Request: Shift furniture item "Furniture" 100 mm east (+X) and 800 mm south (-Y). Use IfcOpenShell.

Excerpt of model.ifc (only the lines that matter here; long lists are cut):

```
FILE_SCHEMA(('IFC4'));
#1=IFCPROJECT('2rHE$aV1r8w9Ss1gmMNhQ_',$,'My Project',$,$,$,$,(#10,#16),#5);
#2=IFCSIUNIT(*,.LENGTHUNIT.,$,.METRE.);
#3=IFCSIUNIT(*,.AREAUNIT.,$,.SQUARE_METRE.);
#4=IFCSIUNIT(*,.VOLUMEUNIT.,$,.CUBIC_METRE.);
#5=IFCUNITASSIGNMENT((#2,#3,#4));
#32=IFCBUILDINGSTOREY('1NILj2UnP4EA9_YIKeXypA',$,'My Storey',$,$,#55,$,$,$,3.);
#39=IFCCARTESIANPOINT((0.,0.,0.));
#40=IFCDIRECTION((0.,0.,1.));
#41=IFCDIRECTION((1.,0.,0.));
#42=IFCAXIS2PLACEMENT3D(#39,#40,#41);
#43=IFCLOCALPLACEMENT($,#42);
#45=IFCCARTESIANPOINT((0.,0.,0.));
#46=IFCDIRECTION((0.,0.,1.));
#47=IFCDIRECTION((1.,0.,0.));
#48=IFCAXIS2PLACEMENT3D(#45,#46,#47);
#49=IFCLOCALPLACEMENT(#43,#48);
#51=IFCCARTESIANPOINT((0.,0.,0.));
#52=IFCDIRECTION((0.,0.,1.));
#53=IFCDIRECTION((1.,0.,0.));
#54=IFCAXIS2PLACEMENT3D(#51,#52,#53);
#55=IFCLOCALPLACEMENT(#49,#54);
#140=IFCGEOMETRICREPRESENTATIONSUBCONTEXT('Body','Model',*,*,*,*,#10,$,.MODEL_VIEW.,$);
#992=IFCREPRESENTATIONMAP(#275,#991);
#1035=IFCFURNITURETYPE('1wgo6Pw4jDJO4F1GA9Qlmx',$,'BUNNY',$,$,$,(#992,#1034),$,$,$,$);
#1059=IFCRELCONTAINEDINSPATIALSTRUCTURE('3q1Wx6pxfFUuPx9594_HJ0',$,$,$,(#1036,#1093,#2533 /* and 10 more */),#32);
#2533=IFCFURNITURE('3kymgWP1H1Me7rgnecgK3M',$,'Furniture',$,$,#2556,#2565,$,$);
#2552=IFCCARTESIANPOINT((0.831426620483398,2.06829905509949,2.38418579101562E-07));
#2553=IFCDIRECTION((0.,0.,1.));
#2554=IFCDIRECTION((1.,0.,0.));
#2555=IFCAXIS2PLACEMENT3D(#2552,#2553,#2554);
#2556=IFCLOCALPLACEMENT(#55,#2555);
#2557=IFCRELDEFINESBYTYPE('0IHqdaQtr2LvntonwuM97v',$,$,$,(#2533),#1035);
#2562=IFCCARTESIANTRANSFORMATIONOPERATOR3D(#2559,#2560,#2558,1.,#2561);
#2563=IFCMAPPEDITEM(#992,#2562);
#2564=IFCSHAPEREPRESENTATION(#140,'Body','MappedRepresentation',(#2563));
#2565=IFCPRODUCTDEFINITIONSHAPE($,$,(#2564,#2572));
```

```python
import ifcopenshell
import ifcopenshell.api.geometry
import ifcopenshell.util.placement

model = ifcopenshell.open("model.ifc")

item = model.by_id(2533)
matrix = ifcopenshell.util.placement.get_local_placement(item.ObjectPlacement)
matrix[0, 3] += 0.1
matrix[1, 3] -= 0.8
ifcopenshell.api.geometry.edit_object_placement(model, product=item, matrix=matrix, is_si=False)

print(ifcopenshell.util.placement.get_local_placement(item.ObjectPlacement).round(3) + 0.0)

model.write("model_v2.ifc")
```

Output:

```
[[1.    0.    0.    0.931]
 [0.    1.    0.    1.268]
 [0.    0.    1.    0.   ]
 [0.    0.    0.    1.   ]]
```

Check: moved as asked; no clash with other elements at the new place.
